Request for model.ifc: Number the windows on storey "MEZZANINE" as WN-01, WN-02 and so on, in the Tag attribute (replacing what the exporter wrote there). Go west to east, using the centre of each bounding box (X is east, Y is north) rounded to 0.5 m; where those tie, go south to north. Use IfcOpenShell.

First a look at what the model holds.

```python
import ifcopenshell
import ifcopenshell.util.element
import ifcopenshell.util.placement

model = ifcopenshell.open("model.ifc")
print(model.schema)
storey = next(s for s in model.by_type("IfcBuildingStorey") if s.Name == "MEZZANINE")
windows = [e for e in ifcopenshell.util.element.get_decomposition(storey) if e.is_a("IfcWindow")]
for e in sorted(windows, key=lambda e: e.id()):
    origin = ifcopenshell.util.placement.get_local_placement(e.ObjectPlacement)[:3, 3]
    print(e.id(), e.Tag, e.Name, origin.round(2) + 0.0, sep=" | ")
```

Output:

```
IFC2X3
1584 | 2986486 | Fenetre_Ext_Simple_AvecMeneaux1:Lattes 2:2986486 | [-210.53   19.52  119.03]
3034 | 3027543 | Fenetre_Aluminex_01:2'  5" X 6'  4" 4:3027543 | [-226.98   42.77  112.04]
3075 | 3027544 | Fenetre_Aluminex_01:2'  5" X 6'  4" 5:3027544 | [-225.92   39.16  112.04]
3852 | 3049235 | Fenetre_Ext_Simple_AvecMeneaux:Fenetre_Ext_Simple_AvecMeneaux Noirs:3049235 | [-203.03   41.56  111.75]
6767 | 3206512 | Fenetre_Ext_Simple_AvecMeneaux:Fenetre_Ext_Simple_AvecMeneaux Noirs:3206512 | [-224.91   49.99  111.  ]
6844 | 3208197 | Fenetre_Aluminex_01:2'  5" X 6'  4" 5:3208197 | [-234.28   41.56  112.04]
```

```python
import ifcopenshell
import ifcopenshell.geom
import ifcopenshell.util.element
import ifcopenshell.util.shape

model = ifcopenshell.open("model.ifc")
settings = ifcopenshell.geom.settings()
settings.set("use-world-coords", True)


def centre(element):
    shape = ifcopenshell.geom.create_shape(settings, element)
    return ifcopenshell.util.shape.get_bbox_centroid(shape.geometry)


storey = next(s for s in model.by_type("IfcBuildingStorey") if s.Name == "MEZZANINE")
windows = [e for e in ifcopenshell.util.element.get_decomposition(storey) if e.is_a("IfcWindow")]

# Insertion points can sit at a corner or the storey origin, so sort by the geometry (in metres).
centres = {e: centre(e) for e in windows}
windows.sort(key=lambda e: (round(centres[e][0] / 0.5), centres[e][1]))

for i, e in enumerate(windows, start=1):
    number = f"WN-{i:02d}"
    e.Tag = number
    print(e.id(), number)

model.write("model-out.ifc")
```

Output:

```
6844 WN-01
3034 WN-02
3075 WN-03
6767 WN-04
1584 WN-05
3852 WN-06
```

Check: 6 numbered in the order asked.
